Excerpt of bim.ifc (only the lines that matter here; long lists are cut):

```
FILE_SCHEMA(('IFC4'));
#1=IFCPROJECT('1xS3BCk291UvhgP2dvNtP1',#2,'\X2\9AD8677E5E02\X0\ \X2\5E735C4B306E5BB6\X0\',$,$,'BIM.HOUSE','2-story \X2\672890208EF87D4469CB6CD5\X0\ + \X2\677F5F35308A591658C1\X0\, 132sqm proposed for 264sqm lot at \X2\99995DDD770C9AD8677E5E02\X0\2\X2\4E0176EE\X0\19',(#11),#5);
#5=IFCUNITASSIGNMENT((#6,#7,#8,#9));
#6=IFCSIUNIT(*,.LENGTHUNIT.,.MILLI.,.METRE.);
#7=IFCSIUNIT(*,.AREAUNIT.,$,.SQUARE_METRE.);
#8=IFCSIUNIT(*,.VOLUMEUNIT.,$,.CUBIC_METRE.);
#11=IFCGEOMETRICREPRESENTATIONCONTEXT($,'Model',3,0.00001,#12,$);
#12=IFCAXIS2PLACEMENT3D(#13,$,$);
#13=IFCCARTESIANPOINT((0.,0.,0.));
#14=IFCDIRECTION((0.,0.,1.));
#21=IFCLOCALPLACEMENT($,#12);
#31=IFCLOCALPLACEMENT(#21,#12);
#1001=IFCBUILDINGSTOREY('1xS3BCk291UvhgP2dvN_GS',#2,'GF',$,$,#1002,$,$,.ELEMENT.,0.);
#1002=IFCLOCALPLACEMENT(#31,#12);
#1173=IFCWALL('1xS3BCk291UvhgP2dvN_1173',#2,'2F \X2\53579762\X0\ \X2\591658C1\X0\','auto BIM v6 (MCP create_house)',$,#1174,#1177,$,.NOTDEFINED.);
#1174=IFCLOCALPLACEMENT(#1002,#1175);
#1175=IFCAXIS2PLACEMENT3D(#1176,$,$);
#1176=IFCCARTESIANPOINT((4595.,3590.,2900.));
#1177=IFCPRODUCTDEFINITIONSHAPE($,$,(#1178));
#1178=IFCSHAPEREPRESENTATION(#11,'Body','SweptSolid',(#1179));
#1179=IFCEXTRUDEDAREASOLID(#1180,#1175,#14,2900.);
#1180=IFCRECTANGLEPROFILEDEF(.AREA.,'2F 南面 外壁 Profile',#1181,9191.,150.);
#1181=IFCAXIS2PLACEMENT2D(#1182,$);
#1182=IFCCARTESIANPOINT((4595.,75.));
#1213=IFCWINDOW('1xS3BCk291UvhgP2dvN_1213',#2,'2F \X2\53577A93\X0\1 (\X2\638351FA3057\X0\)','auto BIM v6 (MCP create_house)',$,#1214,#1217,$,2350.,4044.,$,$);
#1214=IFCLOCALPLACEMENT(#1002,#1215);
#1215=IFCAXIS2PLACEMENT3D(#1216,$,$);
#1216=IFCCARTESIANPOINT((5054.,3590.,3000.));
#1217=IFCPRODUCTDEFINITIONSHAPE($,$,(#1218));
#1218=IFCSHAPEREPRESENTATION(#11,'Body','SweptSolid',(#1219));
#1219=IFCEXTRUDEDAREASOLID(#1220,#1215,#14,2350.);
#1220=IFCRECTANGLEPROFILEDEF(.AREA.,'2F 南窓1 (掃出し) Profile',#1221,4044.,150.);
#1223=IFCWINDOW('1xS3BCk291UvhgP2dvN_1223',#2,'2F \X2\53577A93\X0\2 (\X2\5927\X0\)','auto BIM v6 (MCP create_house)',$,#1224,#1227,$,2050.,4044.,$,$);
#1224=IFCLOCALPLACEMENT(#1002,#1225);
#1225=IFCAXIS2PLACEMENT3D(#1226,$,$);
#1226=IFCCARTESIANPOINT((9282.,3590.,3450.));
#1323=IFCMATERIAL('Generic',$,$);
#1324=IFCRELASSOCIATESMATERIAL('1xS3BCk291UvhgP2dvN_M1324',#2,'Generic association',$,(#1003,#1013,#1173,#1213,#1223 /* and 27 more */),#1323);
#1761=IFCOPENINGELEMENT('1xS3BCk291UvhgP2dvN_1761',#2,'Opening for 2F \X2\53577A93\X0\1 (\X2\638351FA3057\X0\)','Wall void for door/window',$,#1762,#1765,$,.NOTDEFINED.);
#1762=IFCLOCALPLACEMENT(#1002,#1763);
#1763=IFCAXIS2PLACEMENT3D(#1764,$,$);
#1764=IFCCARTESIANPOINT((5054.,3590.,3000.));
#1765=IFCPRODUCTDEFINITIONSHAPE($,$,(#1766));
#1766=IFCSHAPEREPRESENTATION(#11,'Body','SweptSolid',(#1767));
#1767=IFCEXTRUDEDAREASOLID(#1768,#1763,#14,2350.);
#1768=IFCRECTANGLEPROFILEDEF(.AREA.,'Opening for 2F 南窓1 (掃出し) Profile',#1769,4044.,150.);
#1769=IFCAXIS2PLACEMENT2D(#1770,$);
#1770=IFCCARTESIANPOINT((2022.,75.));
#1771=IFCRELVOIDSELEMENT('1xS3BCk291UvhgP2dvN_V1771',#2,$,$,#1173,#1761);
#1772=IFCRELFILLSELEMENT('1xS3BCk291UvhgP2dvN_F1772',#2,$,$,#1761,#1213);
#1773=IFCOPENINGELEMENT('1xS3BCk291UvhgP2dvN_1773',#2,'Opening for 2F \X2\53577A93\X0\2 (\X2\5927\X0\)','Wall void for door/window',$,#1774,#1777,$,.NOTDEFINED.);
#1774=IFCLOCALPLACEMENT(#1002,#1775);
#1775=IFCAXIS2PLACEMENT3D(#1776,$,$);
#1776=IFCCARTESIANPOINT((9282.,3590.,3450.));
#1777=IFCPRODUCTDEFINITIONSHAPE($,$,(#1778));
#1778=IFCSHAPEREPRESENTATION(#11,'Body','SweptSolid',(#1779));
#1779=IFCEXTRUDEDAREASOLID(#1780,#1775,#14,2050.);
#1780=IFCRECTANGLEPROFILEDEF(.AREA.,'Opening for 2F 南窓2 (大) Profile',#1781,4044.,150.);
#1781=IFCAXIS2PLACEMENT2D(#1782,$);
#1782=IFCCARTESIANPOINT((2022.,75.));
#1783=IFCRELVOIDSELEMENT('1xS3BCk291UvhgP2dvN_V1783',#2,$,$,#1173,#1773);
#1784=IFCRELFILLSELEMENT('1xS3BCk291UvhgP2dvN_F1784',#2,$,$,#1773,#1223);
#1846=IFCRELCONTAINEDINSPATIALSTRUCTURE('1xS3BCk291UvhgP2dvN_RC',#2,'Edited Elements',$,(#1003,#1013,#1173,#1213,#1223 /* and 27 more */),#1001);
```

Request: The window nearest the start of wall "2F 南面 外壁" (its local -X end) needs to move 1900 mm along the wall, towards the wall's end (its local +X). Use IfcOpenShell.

```python
import ifcopenshell
import ifcopenshell.api.geometry
import ifcopenshell.util.placement

model = ifcopenshell.open("bim.ifc")

window = model.by_guid("1xS3BCk291UvhgP2dvN_1213")
opening = window.FillsVoids[0].RelatingOpeningElement
wall = opening.VoidsElements[0].RelatingBuildingElement

wall_matrix = ifcopenshell.util.placement.get_local_placement(wall.ObjectPlacement)
shift = wall_matrix[:3, 0] * 1900.0
before = ifcopenshell.util.placement.get_local_placement(window.ObjectPlacement)[:3, 3].copy()

# The window is not placed relative to its opening, so move both.
for product in (opening, window):
    matrix = ifcopenshell.util.placement.get_local_placement(product.ObjectPlacement)
    matrix[:3, 3] += shift
    ifcopenshell.api.geometry.edit_object_placement(model, product=product, matrix=matrix, is_si=False)

after = ifcopenshell.util.placement.get_local_placement(window.ObjectPlacement)[:3, 3]
print("window moved by", (after - before).round(3) + 0.0)

model.write("bim_rev.ifc")
```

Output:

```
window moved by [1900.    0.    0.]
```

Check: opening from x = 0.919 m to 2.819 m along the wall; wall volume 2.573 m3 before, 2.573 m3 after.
